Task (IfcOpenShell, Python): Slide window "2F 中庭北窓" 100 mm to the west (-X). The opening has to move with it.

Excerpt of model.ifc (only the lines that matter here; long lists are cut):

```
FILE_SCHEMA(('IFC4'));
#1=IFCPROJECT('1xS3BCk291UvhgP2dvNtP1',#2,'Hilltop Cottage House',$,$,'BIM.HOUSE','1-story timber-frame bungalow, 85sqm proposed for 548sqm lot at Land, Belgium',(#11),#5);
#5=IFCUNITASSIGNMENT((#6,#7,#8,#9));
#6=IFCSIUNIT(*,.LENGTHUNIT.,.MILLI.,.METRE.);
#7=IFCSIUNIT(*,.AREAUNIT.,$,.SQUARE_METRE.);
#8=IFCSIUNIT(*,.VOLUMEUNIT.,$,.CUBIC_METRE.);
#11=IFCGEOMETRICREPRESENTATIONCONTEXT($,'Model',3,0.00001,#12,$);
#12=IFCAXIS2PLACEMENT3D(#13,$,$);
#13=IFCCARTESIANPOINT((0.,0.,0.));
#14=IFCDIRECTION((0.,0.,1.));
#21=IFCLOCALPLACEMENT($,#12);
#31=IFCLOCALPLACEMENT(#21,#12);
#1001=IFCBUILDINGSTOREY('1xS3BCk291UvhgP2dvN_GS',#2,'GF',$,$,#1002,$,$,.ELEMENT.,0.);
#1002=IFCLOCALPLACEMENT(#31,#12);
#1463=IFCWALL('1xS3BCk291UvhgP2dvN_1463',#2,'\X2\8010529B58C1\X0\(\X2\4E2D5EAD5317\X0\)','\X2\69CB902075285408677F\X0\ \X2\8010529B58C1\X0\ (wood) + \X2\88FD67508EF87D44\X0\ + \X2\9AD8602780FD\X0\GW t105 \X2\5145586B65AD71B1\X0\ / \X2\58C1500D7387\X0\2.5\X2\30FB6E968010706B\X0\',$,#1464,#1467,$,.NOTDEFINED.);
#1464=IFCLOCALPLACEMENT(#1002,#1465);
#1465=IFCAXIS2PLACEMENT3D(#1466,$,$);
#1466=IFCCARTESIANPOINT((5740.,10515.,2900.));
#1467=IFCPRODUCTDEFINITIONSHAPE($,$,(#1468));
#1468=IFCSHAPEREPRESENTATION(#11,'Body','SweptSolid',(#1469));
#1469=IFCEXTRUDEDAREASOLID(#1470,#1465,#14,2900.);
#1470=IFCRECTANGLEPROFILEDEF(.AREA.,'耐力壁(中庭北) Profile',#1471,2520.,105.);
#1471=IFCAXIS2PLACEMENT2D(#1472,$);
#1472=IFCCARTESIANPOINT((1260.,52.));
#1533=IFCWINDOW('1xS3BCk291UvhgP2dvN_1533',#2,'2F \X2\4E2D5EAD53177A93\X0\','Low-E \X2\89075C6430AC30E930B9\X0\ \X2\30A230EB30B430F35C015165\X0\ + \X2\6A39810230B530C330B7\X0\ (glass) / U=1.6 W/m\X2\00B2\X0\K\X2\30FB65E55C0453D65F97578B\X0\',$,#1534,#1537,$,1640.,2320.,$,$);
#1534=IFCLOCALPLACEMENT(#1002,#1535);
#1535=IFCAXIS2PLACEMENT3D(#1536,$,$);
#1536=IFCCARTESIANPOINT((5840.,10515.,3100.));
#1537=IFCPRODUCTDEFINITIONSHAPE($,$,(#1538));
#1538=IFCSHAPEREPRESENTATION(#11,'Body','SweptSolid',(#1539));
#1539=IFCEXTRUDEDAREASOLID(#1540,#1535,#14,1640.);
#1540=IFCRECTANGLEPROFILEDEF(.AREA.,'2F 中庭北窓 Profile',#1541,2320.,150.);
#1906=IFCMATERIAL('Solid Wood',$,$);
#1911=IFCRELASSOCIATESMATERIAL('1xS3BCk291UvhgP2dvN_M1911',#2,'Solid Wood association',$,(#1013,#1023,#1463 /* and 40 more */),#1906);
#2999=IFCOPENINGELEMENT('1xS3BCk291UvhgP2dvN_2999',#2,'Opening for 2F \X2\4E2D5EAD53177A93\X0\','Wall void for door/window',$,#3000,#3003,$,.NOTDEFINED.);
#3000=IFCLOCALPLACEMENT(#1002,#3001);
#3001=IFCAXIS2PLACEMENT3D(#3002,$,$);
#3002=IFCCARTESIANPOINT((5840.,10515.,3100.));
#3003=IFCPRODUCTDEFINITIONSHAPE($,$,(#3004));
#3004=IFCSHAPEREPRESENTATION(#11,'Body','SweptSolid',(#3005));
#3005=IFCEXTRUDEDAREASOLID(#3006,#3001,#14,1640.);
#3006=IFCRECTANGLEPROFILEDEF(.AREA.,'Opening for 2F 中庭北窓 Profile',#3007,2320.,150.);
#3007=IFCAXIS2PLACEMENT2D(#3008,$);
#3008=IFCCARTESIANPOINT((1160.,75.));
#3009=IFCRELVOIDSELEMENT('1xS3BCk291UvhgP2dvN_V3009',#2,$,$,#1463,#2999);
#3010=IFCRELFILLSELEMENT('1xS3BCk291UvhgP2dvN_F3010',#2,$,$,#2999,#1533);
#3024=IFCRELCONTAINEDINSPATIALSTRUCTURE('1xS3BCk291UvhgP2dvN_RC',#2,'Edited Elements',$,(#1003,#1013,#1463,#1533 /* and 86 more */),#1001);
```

```python
import ifcopenshell
import ifcopenshell.api.geometry
import ifcopenshell.util.placement

model = ifcopenshell.open("model.ifc")

window = model.by_guid("1xS3BCk291UvhgP2dvN_1533")
opening = window.FillsVoids[0].RelatingOpeningElement
wall = opening.VoidsElements[0].RelatingBuildingElement

wall_matrix = ifcopenshell.util.placement.get_local_placement(wall.ObjectPlacement)
shift = wall_matrix[:3, 0] * -100.0
before = ifcopenshell.util.placement.get_local_placement(window.ObjectPlacement)[:3, 3].copy()

# The window is not placed relative to its opening, so move both.
for product in (opening, window):
    matrix = ifcopenshell.util.placement.get_local_placement(product.ObjectPlacement)
    matrix[:3, 3] += shift
    ifcopenshell.api.geometry.edit_object_placement(model, product=product, matrix=matrix, is_si=False)

after = ifcopenshell.util.placement.get_local_placement(window.ObjectPlacement)[:3, 3]
print("window moved by", (after - before).round(3) + 0.0)

model.write("model_updated.ifc")
```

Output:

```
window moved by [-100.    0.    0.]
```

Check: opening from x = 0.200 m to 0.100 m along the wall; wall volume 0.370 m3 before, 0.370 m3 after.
